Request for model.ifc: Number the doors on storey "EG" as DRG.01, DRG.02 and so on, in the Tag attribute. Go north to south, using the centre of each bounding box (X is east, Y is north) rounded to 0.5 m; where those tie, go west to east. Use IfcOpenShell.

First a look at what the model holds.

```python
import ifcopenshell
import ifcopenshell.util.element
import ifcopenshell.util.placement

model = ifcopenshell.open("model.ifc")
print(model.schema)
storey = next(s for s in model.by_type("IfcBuildingStorey") if s.Name == "EG")
doors = [e for e in ifcopenshell.util.element.get_decomposition(storey) if e.is_a("IfcDoor")]
for e in sorted(doors, key=lambda e: e.id()):
    origin = ifcopenshell.util.placement.get_local_placement(e.ObjectPlacement)[:3, 3]
    print(e.id(), e.Tag, e.Name, origin.round(2) + 0.0, sep=" | ")
```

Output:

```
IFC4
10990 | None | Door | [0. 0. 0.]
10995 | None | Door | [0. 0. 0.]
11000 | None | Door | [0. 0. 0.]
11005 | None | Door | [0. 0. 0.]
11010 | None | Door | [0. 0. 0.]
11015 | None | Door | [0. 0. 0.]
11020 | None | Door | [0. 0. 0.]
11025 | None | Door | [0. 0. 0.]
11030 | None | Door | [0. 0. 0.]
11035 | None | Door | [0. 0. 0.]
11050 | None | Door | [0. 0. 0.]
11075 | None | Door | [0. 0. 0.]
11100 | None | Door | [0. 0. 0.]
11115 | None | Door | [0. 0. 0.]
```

```python
import ifcopenshell
import ifcopenshell.geom
import ifcopenshell.util.element
import ifcopenshell.util.shape

model = ifcopenshell.open("model.ifc")
settings = ifcopenshell.geom.settings()
settings.set("use-world-coords", True)


def centre(element):
    shape = ifcopenshell.geom.create_shape(settings, element)
    return ifcopenshell.util.shape.get_bbox_centroid(shape.geometry)


storey = next(s for s in model.by_type("IfcBuildingStorey") if s.Name == "EG")
doors = [e for e in ifcopenshell.util.element.get_decomposition(storey) if e.is_a("IfcDoor")]

# Insertion points can sit at a corner or the storey origin, so sort by the geometry (in metres).
centres = {e: centre(e) for e in doors}
doors.sort(key=lambda e: (-round(centres[e][1] / 0.5), centres[e][0]))

for i, e in enumerate(doors, start=1):
    number = f"DRG.{i:02d}"
    e.Tag = number
    print(e.id(), number)

model.write("model_rev.ifc")
```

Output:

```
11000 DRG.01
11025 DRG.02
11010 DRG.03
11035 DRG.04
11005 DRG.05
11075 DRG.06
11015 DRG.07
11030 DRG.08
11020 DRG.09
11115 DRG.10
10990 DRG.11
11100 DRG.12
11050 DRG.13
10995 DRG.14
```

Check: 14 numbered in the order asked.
